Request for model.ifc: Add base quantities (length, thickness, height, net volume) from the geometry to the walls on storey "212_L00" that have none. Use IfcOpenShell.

First a look at what the model holds.

```python
import ifcopenshell
import ifcopenshell.util.element
import ifcopenshell.util.unit

model = ifcopenshell.open("model.ifc")
print(model.schema)
for unit_type in ("LENGTHUNIT", "AREAUNIT", "VOLUMEUNIT"):
    print(unit_type, ifcopenshell.util.unit.calculate_unit_scale(model, unit_type))
storey = next(s for s in model.by_type("IfcBuildingStorey") if s.Name == "212_L00")
walls = [e for e in ifcopenshell.util.element.get_decomposition(storey) if e.is_a("IfcWall")]
for e in sorted(walls, key=lambda e: e.id()):
    print(e.id(), e.is_a(), e.Name, list(ifcopenshell.util.element.get_psets(e, qtos_only=True)), sep=" | ")
```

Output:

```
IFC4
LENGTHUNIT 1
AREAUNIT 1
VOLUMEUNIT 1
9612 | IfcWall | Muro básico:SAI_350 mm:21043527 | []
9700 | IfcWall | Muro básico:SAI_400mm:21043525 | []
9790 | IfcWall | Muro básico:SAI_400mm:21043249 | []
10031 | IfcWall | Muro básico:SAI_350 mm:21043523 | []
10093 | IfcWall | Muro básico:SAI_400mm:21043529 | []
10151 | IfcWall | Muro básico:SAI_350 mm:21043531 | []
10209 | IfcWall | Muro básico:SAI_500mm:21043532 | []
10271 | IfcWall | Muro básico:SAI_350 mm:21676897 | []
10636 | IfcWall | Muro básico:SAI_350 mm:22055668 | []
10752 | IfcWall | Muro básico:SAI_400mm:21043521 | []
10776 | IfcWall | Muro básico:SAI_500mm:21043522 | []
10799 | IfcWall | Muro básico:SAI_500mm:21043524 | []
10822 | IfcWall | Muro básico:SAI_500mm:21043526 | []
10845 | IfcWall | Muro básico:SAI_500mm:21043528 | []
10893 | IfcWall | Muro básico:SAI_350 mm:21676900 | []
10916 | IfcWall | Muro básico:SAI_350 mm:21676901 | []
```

```python
import ifcopenshell
import ifcopenshell.api.pset
import ifcopenshell.geom
import ifcopenshell.util.element
import ifcopenshell.util.shape
import ifcopenshell.util.unit

model = ifcopenshell.open("model.ifc")
unit_scale = ifcopenshell.util.unit.calculate_unit_scale(model)
volume_scale = ifcopenshell.util.unit.calculate_unit_scale(model, "VOLUMEUNIT")
settings = ifcopenshell.geom.settings()

storey = next(s for s in model.by_type("IfcBuildingStorey") if s.Name == "212_L00")
walls = [e for e in ifcopenshell.util.element.get_decomposition(storey) if e.is_a("IfcWall")]

for e in sorted(walls, key=lambda e: e.id()):
    if ifcopenshell.util.element.get_psets(e, qtos_only=True, should_inherit=False):
        continue
    # Geometry comes back in metres, in the element's own axes.
    shape = ifcopenshell.geom.create_shape(settings, e)
    values = {
        "Length": ifcopenshell.util.shape.get_x(shape.geometry) / unit_scale,
        "Width": ifcopenshell.util.shape.get_y(shape.geometry) / unit_scale,
        "Height": ifcopenshell.util.shape.get_z(shape.geometry) / unit_scale,
        "NetVolume": ifcopenshell.util.shape.get_volume(shape.geometry) / volume_scale,
    }
    qto = ifcopenshell.api.pset.add_qto(model, product=e, name="Qto_WallBaseQuantities")
    ifcopenshell.api.pset.edit_qto(model, qto=qto, properties=values)
    print(e.id(), {k: round(v, 3) for k, v in values.items()})

model.write("model_rev.ifc")
```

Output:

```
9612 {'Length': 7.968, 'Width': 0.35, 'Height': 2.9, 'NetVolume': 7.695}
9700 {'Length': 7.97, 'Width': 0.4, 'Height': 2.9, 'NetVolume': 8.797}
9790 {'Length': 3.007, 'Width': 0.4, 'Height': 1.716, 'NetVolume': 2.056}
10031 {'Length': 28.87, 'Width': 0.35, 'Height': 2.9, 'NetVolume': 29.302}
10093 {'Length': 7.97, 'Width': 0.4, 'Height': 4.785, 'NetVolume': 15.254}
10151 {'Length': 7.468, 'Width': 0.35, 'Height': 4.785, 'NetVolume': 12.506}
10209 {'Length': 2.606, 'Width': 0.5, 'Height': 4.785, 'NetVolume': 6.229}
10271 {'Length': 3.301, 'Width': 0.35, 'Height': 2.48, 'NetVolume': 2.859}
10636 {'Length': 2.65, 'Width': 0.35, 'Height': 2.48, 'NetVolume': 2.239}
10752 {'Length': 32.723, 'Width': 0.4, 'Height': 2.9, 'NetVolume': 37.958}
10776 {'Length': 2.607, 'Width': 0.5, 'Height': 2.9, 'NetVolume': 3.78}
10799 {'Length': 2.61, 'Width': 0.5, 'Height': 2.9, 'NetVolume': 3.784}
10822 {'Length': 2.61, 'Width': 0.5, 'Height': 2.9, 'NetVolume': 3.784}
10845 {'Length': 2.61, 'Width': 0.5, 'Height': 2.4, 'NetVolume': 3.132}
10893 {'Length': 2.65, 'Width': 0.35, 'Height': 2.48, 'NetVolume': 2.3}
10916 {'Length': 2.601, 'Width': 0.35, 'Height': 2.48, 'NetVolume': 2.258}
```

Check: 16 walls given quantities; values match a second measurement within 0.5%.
